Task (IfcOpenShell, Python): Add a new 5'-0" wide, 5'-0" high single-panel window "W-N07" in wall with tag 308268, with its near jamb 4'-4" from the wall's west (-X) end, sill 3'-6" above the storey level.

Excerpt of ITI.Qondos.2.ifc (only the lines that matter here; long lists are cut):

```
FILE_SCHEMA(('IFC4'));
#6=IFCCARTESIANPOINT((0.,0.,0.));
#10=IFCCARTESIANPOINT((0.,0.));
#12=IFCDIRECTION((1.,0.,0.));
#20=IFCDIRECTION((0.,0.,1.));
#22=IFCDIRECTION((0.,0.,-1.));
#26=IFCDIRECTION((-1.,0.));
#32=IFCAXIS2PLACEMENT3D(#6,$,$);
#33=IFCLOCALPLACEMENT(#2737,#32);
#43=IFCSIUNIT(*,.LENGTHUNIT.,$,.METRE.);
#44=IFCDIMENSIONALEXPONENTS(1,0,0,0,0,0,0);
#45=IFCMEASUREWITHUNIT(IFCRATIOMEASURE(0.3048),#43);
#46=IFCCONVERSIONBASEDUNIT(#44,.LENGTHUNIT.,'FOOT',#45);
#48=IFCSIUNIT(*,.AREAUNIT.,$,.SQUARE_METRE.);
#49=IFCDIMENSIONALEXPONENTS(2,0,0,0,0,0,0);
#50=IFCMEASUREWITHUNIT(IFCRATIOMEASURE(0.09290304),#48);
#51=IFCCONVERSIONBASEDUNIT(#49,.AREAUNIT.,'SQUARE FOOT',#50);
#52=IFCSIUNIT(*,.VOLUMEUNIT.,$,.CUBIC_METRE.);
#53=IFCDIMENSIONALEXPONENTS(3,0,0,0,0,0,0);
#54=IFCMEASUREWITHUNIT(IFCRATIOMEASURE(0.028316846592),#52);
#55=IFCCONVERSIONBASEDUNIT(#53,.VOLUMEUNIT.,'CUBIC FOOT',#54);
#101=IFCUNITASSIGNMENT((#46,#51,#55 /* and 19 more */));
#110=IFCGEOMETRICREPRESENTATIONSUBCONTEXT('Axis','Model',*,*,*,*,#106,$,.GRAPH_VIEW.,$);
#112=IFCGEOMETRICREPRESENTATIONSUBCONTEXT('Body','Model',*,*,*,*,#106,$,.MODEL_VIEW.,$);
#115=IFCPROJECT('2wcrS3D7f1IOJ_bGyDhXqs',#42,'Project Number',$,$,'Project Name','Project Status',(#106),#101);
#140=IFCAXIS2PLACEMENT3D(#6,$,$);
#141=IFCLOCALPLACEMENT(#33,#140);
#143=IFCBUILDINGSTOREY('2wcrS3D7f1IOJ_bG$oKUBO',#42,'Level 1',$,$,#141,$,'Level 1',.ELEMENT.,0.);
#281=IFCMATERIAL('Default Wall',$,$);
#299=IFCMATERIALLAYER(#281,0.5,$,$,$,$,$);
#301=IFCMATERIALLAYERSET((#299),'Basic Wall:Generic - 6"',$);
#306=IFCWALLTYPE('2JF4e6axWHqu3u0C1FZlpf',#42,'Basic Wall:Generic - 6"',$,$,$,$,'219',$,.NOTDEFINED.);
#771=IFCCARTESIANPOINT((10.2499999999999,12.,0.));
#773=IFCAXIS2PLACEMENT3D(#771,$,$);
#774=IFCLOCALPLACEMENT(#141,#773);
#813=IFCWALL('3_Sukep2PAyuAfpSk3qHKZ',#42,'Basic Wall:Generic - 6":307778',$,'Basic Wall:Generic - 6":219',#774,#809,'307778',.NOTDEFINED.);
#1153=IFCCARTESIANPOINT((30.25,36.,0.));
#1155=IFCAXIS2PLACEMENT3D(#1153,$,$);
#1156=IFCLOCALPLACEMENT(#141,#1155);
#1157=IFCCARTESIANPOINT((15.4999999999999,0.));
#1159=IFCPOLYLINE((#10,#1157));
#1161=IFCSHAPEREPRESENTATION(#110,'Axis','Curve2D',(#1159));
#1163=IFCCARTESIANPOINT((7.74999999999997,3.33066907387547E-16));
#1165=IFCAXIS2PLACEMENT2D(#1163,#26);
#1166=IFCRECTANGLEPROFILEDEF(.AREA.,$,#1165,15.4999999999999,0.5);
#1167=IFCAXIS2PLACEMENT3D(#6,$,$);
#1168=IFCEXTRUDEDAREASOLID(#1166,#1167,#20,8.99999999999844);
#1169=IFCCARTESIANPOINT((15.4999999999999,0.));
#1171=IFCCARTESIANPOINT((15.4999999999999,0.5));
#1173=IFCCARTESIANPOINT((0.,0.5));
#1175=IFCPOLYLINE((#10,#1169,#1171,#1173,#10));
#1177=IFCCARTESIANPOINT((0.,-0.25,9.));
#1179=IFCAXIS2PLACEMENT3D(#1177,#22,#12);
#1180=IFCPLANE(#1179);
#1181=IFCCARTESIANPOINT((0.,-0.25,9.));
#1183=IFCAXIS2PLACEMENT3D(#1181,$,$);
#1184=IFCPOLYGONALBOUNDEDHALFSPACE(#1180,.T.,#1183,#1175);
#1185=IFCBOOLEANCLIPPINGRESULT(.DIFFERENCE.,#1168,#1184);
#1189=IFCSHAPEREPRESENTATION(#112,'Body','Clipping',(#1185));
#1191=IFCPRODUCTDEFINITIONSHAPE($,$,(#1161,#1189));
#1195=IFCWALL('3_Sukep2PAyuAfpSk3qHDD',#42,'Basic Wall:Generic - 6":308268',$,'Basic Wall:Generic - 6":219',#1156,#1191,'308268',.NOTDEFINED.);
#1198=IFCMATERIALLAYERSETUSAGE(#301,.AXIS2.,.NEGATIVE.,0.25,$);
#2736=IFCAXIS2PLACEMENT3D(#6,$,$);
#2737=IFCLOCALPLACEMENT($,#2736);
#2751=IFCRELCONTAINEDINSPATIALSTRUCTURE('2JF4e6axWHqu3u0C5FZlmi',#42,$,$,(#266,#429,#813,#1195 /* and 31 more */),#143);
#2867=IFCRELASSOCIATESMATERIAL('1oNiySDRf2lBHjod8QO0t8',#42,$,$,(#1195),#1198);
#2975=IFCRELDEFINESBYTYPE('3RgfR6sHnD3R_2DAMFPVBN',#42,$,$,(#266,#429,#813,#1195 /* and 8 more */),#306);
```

```python
import numpy as np
import ifcopenshell
import ifcopenshell.api.feature
import ifcopenshell.api.geometry
import ifcopenshell.api.root
import ifcopenshell.api.spatial
import ifcopenshell.geom
import ifcopenshell.util.element
import ifcopenshell.util.placement
import ifcopenshell.util.representation
import ifcopenshell.util.shape
import ifcopenshell.util.unit

model = ifcopenshell.open("ITI.Qondos.2.ifc")
unit_scale = ifcopenshell.util.unit.calculate_unit_scale(model)
settings = ifcopenshell.geom.settings()


def volume(element):
    """Net volume in cubic metres, openings subtracted."""
    shape = ifcopenshell.geom.create_shape(settings, element)
    return ifcopenshell.util.shape.get_volume(shape.geometry)


wall = model.by_guid("3_Sukep2PAyuAfpSk3qHDD")
storey = ifcopenshell.util.element.get_container(wall, ifc_class="IfcBuildingStorey")
context = ifcopenshell.util.representation.get_context(model, "Model", "Body", "MODEL_VIEW")
before = volume(wall)

width, height, from_end, sill = 1.524, 1.524, 1.3208, 1.0668  # metres

# The wall runs along its own X axis, and the end named is its -X end.
wall_shape = ifcopenshell.geom.create_shape(settings, wall)
x, y, z = ifcopenshell.util.shape.get_vertices(wall_shape.geometry).T
start = x.min() + from_end
face, thickness = float(y.min()), float(y.max() - y.min())
wall_matrix = ifcopenshell.util.placement.get_local_placement(wall.ObjectPlacement)
level = ifcopenshell.util.placement.get_local_placement(storey.ObjectPlacement)[2, 3]


def in_wall(x, y):
    """Placement at x, y metres in the wall's axes, at sill height."""
    matrix = wall_matrix.copy()
    matrix[:, 3] = wall_matrix @ np.array([x / unit_scale, y / unit_scale, 0.0, 1.0])
    matrix[2, 3] = level + sill / unit_scale
    return matrix


# Opening: a box that overshoots both wall faces by 50 mm.
opening = ifcopenshell.api.root.create_entity(model, ifc_class="IfcOpeningElement", predefined_type="OPENING")
box = ifcopenshell.api.geometry.add_wall_representation(
    model, context=context, length=width, height=height, thickness=thickness + 0.1
)
ifcopenshell.api.geometry.assign_representation(model, product=opening, representation=box)
ifcopenshell.api.geometry.edit_object_placement(model, product=opening, matrix=in_wall(start, face - 0.05), is_si=False)
ifcopenshell.api.feature.add_feature(model, feature=opening, element=wall)

window = ifcopenshell.api.root.create_entity(model, ifc_class="IfcWindow", name="W-N07", predefined_type="WINDOW")
window.OverallWidth, window.OverallHeight = width / unit_scale, height / unit_scale
window.PartitioningType = "SINGLE_PANEL"
body = ifcopenshell.api.geometry.add_window_representation(
    model,
    context=context,
    overall_width=window.OverallWidth,
    overall_height=window.OverallHeight,
    partition_type="SINGLE_PANEL",
)
ifcopenshell.api.geometry.assign_representation(model, product=window, representation=body)
ifcopenshell.api.spatial.assign_container(model, products=[window], relating_structure=storey)
ifcopenshell.api.feature.add_filling(model, opening=opening, element=window)

# Centre the window in the wall's thickness.
ifcopenshell.api.geometry.edit_object_placement(model, product=window, matrix=in_wall(start, face), is_si=False)
window_shape = ifcopenshell.geom.create_shape(settings, window)
depth = ifcopenshell.util.shape.get_vertices(window_shape.geometry)[:, 1]
offset = face + thickness / 2 - (depth.min() + depth.max()) / 2
ifcopenshell.api.geometry.edit_object_placement(model, product=window, matrix=in_wall(start, offset), is_si=False)

after = volume(wall)

print(f"wall volume {before:.3f} -> {after:.3f} m3")

model.write("ITI.Qondos.2-out.ifc")
```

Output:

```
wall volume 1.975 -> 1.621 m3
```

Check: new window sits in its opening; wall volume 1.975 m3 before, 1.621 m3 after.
